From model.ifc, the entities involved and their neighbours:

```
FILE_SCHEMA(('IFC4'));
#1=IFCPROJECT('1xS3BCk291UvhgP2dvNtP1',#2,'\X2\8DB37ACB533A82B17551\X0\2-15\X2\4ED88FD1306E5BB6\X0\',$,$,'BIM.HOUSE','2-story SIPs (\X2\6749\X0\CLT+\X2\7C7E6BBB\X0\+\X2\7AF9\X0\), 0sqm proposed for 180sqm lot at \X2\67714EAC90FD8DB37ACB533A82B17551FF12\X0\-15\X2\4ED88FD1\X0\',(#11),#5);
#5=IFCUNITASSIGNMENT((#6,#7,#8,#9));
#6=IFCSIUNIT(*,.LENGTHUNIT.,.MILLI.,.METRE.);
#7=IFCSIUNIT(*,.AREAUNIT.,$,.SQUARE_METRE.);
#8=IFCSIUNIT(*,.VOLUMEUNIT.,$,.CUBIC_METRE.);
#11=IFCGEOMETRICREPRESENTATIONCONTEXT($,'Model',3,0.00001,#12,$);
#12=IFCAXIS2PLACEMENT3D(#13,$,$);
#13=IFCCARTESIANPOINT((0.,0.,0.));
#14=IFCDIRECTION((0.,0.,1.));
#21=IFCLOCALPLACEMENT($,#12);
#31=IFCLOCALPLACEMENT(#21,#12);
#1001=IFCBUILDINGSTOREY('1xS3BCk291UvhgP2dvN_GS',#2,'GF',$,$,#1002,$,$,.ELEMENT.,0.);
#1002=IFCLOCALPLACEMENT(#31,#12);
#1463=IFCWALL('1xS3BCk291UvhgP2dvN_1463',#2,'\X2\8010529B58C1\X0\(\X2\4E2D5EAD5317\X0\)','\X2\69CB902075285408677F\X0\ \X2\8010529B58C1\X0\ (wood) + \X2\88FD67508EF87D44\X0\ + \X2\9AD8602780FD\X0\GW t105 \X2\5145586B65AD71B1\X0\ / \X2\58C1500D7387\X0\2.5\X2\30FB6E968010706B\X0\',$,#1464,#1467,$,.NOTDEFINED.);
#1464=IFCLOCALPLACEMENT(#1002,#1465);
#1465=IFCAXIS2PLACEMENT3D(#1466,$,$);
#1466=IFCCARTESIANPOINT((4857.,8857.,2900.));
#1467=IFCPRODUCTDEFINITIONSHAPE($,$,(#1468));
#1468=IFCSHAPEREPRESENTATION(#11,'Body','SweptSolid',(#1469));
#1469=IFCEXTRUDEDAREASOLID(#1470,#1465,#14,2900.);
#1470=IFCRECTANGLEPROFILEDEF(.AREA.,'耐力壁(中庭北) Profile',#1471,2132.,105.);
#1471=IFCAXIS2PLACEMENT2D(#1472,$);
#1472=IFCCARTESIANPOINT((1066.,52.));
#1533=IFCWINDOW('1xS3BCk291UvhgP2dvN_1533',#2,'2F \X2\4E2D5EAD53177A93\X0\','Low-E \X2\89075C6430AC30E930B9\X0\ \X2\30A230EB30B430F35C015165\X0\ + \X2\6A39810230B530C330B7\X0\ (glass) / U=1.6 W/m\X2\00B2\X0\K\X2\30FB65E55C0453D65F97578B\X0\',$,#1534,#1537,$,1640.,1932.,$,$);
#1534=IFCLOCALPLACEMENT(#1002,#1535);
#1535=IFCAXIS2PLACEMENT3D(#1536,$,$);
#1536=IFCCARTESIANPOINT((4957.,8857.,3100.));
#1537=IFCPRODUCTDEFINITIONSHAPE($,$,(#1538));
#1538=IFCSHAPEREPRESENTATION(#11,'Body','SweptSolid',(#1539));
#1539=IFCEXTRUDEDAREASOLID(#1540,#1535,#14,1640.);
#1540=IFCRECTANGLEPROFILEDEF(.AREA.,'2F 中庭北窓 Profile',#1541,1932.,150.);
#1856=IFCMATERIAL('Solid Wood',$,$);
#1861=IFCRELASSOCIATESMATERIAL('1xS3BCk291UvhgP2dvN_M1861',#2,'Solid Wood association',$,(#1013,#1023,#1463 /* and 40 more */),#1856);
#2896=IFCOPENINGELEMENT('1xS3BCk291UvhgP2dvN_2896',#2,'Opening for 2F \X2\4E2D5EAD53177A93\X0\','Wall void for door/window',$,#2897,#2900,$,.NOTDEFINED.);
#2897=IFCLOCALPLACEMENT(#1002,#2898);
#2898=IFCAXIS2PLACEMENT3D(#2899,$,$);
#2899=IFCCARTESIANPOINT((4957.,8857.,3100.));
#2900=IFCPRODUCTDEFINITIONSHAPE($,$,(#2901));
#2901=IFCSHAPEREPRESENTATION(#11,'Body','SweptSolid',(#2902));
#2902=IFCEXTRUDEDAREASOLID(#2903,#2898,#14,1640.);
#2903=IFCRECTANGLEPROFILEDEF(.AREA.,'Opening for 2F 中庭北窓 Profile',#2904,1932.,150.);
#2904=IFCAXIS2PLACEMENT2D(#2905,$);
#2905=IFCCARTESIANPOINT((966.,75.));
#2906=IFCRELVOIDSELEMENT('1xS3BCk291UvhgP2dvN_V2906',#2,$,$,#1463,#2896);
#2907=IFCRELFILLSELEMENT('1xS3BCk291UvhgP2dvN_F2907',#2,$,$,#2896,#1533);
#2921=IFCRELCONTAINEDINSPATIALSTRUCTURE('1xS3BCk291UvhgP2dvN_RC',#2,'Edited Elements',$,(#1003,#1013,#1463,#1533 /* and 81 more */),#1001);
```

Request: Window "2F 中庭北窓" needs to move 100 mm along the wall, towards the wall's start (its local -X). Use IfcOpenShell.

```python
import ifcopenshell
import ifcopenshell.api.geometry
import ifcopenshell.util.placement
import ifcopenshell.util.unit

model = ifcopenshell.open("model.ifc")
unit_scale = ifcopenshell.util.unit.calculate_unit_scale(model)

window = model.by_guid("1xS3BCk291UvhgP2dvN_1533")
opening = window.FillsVoids[0].RelatingOpeningElement
wall = opening.VoidsElements[0].RelatingBuildingElement

wall_matrix = ifcopenshell.util.placement.get_local_placement(wall.ObjectPlacement)
shift = wall_matrix[:3, 0] * -0.1 / unit_scale
before = ifcopenshell.util.placement.get_local_placement(window.ObjectPlacement)[:3, 3].copy()

# The window is not placed relative to its opening, so move both.
for product in (opening, window):
    matrix = ifcopenshell.util.placement.get_local_placement(product.ObjectPlacement)
    matrix[:3, 3] += shift
    ifcopenshell.api.geometry.edit_object_placement(model, product=product, matrix=matrix, is_si=False)

after = ifcopenshell.util.placement.get_local_placement(window.ObjectPlacement)[:3, 3]
print("window moved by", (after - before).round(3) + 0.0)

model.write("model_v2.ifc")
```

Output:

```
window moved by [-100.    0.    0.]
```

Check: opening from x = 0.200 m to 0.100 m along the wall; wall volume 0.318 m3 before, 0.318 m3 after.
